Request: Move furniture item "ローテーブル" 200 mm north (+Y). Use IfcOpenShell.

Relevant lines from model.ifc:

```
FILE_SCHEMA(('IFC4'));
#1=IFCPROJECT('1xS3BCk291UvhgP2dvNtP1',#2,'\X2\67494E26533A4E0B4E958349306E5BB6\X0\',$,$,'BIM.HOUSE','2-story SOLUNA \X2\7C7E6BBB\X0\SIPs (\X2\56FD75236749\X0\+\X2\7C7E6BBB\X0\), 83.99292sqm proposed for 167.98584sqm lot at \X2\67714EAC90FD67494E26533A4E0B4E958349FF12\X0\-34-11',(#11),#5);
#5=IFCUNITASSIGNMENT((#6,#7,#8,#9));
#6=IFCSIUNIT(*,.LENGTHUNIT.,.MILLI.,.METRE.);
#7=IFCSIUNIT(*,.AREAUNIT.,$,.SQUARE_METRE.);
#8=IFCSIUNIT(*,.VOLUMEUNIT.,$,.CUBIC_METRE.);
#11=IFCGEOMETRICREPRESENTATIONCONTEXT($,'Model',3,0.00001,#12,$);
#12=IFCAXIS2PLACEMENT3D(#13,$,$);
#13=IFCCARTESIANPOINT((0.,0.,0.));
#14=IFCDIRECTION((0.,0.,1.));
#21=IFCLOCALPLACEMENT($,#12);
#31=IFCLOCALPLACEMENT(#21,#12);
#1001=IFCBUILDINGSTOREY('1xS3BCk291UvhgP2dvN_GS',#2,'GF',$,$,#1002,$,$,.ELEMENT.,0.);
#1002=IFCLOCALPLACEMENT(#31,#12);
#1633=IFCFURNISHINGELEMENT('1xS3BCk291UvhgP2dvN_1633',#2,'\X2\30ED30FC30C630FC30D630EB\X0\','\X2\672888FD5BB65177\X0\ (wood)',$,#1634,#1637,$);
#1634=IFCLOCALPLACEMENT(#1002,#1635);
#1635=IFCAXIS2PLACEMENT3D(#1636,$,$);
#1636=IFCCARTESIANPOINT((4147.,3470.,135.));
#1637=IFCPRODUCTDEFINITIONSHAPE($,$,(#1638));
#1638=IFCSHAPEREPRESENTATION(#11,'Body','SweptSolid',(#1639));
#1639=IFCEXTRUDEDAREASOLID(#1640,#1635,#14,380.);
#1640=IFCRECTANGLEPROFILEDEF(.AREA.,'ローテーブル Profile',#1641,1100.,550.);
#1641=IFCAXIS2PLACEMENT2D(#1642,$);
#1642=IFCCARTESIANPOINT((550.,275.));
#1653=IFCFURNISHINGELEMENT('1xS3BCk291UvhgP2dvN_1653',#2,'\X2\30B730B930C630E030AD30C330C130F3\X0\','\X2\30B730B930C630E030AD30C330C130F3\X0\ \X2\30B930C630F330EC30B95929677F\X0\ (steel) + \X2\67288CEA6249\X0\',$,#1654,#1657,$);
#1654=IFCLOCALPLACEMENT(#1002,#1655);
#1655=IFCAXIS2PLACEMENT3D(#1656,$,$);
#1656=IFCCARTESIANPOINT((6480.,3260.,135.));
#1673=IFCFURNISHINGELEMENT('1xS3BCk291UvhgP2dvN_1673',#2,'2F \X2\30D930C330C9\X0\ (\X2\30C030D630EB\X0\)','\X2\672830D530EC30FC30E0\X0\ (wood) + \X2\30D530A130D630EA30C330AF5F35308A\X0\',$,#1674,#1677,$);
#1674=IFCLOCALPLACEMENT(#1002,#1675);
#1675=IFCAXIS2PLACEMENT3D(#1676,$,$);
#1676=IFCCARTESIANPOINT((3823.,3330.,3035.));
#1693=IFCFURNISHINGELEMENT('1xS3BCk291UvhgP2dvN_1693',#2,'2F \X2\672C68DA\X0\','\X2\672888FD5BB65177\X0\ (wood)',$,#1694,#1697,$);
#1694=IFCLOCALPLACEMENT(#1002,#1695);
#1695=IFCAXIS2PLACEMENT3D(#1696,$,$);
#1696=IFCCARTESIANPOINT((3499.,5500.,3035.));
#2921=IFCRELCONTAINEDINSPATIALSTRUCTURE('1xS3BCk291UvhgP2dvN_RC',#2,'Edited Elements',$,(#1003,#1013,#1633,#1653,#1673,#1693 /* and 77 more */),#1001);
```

```python
import ifcopenshell
import ifcopenshell.api.geometry
import ifcopenshell.util.placement
import ifcopenshell.util.unit

model = ifcopenshell.open("model.ifc")
unit_scale = ifcopenshell.util.unit.calculate_unit_scale(model)

item = model.by_guid("1xS3BCk291UvhgP2dvN_1633")
matrix = ifcopenshell.util.placement.get_local_placement(item.ObjectPlacement)
matrix[1, 3] += 0.2 / unit_scale
ifcopenshell.api.geometry.edit_object_placement(model, product=item, matrix=matrix, is_si=False)

print(ifcopenshell.util.placement.get_local_placement(item.ObjectPlacement).round(3) + 0.0)

model.write("model_updated.ifc")
```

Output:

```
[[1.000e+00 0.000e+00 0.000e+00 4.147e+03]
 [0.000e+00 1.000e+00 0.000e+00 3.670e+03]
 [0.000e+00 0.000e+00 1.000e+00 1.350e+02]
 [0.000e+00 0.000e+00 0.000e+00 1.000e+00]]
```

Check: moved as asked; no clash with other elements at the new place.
